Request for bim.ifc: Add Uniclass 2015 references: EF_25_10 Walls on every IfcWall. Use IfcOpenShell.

First a look at what the model holds.

```python
import ifcopenshell

model = ifcopenshell.open("bim.ifc")
print(model.schema)
print("classifications:", [c.Name for c in model.by_type("IfcClassification")])
for ifc_class in ("IfcDoor", "IfcRoof", "IfcStair", "IfcWall", "IfcWindow"):
    print(ifc_class, len(model.by_type(ifc_class)))
```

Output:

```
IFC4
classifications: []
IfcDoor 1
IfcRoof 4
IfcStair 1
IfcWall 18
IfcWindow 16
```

```python
import ifcopenshell
import ifcopenshell.api.classification

model = ifcopenshell.open("bim.ifc")

system = ifcopenshell.api.classification.add_classification(model, classification="Uniclass 2015")

codes = {
    "IfcWall": ("EF_25_10", "Walls"),
}
for ifc_class, (code, name) in codes.items():
    products = model.by_type(ifc_class)
    ifcopenshell.api.classification.add_reference(
        model, products=products, classification=system, identification=code, name=name
    )
    print(code, len(products))

model.write("bim_edited.ifc")
```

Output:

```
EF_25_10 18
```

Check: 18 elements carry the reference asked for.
